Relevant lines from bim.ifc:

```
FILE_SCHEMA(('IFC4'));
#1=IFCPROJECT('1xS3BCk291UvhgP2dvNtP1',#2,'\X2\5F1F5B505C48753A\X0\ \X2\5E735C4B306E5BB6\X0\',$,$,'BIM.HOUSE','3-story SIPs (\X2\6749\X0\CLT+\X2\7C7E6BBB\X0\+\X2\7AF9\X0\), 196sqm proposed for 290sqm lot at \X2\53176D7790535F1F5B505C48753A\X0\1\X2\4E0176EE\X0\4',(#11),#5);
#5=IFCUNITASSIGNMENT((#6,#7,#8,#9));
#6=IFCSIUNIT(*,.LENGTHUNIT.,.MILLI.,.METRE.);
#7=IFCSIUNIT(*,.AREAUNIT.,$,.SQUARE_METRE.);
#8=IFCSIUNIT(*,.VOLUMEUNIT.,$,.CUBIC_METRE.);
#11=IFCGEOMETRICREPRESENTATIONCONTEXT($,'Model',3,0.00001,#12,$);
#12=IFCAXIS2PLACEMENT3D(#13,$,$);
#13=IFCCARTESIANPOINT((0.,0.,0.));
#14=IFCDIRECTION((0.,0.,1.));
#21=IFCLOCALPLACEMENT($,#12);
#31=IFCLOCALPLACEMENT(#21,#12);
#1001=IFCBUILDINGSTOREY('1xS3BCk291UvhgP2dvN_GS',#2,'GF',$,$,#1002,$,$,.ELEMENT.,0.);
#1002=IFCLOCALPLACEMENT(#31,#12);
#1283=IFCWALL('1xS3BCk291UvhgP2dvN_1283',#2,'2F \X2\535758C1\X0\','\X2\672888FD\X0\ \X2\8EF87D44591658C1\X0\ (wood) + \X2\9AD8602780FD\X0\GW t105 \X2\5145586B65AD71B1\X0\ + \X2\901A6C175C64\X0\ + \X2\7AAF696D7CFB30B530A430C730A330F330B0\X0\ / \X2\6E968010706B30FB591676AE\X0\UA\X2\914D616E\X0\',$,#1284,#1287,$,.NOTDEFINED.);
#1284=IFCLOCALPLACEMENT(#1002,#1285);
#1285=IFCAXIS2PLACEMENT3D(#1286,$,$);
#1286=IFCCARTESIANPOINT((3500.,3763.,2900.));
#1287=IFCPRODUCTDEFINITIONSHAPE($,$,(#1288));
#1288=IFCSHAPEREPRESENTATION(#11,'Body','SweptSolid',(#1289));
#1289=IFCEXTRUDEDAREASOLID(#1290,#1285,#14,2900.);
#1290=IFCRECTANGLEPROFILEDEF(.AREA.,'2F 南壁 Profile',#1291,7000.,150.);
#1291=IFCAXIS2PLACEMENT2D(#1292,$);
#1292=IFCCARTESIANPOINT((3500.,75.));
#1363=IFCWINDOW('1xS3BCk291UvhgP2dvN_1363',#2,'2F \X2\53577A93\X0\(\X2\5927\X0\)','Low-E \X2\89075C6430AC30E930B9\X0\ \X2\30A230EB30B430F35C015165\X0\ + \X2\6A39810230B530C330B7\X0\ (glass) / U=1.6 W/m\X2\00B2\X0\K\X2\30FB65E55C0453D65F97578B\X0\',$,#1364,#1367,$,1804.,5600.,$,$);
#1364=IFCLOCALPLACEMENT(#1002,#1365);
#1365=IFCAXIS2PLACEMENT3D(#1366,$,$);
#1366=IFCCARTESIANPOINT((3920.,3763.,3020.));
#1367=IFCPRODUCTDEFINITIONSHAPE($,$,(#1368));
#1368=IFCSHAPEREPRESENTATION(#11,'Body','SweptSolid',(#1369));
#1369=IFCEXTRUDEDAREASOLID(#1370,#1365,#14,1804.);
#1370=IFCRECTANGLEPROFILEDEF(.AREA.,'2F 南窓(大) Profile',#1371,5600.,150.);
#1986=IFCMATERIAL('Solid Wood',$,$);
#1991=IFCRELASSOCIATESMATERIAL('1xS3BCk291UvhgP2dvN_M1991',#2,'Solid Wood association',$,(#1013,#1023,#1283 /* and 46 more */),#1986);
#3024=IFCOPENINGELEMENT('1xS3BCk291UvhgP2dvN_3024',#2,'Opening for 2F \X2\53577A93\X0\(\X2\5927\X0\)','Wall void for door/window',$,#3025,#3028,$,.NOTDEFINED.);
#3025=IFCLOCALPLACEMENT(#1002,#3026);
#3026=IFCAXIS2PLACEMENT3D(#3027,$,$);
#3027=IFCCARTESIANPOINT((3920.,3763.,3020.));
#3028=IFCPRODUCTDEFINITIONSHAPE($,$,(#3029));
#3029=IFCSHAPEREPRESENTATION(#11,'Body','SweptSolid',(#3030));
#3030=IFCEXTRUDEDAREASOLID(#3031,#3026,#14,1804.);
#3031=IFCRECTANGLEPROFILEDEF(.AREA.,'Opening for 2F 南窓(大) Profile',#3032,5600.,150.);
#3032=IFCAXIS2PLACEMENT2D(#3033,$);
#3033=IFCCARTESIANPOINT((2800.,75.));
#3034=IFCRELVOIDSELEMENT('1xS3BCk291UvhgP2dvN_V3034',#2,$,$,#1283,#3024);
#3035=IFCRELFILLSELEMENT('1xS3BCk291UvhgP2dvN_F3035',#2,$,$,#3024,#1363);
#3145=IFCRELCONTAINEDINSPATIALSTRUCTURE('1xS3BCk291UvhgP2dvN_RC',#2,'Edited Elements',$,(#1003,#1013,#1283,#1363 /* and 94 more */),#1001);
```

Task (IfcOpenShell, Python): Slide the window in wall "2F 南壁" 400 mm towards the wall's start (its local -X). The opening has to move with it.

```python
import ifcopenshell
import ifcopenshell.api.geometry
import ifcopenshell.util.placement
import ifcopenshell.util.unit

model = ifcopenshell.open("bim.ifc")
unit_scale = ifcopenshell.util.unit.calculate_unit_scale(model)

window = model.by_guid("1xS3BCk291UvhgP2dvN_1363")
opening = window.FillsVoids[0].RelatingOpeningElement
wall = opening.VoidsElements[0].RelatingBuildingElement

wall_matrix = ifcopenshell.util.placement.get_local_placement(wall.ObjectPlacement)
shift = wall_matrix[:3, 0] * -0.4 / unit_scale
before = ifcopenshell.util.placement.get_local_placement(window.ObjectPlacement)[:3, 3].copy()

# The window is not placed relative to its opening, so move both.
for product in (opening, window):
    matrix = ifcopenshell.util.placement.get_local_placement(product.ObjectPlacement)
    matrix[:3, 3] += shift
    ifcopenshell.api.geometry.edit_object_placement(model, product=product, matrix=matrix, is_si=False)

after = ifcopenshell.util.placement.get_local_placement(window.ObjectPlacement)[:3, 3]
print("window moved by", (after - before).round(3) + 0.0)

model.write("bim_edited.ifc")
```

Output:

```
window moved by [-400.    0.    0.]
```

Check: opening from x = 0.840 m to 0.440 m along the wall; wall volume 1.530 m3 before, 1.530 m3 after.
